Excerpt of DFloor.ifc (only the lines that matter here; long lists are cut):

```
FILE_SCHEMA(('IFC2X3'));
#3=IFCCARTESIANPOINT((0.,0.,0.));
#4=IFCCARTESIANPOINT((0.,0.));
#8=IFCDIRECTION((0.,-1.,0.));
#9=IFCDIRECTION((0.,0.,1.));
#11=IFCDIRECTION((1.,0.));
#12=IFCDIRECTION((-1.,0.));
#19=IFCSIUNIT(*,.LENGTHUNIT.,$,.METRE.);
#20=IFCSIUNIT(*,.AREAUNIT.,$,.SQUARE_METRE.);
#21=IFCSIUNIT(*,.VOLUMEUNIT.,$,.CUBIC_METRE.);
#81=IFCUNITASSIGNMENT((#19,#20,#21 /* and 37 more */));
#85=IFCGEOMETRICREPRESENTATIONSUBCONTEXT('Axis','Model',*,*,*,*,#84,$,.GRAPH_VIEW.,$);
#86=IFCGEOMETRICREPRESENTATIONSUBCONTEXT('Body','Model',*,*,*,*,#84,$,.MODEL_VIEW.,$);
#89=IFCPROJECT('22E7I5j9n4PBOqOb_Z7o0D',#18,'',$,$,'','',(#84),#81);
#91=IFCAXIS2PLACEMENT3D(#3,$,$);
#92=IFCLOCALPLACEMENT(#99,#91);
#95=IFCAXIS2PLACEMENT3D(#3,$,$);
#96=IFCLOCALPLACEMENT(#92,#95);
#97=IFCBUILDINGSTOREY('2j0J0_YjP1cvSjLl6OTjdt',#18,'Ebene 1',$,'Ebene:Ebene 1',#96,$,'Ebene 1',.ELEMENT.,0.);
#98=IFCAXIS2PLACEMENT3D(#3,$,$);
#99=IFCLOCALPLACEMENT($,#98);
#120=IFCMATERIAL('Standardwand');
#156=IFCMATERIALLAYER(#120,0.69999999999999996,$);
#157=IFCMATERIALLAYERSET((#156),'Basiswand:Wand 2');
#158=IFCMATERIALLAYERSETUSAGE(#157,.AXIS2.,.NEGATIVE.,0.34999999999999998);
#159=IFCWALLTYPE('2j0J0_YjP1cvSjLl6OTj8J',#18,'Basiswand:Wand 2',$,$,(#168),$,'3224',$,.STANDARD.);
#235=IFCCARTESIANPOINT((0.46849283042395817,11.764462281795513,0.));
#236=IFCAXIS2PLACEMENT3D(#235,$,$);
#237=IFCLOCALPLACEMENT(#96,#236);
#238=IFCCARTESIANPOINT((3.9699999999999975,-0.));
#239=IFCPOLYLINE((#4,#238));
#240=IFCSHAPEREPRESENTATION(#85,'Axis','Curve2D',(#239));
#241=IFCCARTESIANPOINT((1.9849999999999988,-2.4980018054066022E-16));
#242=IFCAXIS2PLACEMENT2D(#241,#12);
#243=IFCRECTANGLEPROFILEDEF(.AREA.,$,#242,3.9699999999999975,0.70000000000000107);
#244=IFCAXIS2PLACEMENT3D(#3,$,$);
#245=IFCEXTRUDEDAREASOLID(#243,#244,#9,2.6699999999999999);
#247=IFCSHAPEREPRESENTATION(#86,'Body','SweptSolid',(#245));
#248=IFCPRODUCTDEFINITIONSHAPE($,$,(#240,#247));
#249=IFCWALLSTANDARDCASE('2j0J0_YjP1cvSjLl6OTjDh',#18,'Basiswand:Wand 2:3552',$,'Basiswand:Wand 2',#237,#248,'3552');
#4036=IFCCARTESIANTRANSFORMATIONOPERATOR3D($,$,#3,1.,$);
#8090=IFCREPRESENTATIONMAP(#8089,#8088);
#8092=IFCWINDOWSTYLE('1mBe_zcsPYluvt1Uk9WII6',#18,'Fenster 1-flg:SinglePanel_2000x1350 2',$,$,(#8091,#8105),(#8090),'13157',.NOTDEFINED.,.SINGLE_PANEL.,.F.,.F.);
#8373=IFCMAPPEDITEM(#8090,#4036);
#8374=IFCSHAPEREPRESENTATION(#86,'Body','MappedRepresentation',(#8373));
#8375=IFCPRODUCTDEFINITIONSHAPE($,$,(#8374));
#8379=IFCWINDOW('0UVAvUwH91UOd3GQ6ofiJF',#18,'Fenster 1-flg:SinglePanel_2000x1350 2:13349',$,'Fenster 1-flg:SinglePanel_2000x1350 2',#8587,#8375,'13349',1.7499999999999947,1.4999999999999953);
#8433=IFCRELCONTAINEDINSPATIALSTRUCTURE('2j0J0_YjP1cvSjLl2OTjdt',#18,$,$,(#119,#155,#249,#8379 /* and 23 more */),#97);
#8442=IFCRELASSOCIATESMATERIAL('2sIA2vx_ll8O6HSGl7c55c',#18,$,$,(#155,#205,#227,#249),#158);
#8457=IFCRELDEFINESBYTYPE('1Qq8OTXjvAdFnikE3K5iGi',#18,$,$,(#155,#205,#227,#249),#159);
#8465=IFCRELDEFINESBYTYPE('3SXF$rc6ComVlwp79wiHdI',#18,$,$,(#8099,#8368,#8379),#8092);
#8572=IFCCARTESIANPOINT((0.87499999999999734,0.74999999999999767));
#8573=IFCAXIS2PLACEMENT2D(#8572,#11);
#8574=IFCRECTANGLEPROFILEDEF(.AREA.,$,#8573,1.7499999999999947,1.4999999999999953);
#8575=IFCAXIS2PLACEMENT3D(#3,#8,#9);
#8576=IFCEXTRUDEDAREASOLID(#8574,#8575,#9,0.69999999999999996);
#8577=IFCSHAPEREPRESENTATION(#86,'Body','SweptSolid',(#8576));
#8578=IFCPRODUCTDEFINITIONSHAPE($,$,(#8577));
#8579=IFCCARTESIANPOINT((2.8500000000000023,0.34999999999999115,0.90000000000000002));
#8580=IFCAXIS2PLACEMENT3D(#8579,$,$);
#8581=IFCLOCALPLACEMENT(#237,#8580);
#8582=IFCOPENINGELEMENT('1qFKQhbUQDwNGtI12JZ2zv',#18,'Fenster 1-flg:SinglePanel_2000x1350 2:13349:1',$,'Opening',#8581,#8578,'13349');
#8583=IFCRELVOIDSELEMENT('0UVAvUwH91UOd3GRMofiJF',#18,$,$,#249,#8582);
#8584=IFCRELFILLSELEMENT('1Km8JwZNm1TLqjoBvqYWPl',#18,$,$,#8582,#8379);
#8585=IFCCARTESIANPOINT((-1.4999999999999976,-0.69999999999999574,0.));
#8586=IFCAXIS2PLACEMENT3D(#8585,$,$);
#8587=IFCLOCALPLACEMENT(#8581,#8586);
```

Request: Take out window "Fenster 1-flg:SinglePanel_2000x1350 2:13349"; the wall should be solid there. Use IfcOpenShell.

```python
import ifcopenshell
import ifcopenshell.api.feature
import ifcopenshell.api.root
import ifcopenshell.geom
import ifcopenshell.util.shape

model = ifcopenshell.open("DFloor.ifc")
settings = ifcopenshell.geom.settings()


def volume(element):
    """Net volume in cubic metres, openings subtracted."""
    shape = ifcopenshell.geom.create_shape(settings, element)
    return ifcopenshell.util.shape.get_volume(shape.geometry)


window = model.by_guid("0UVAvUwH91UOd3GQ6ofiJF")
opening = window.FillsVoids[0].RelatingOpeningElement
wall = opening.VoidsElements[0].RelatingBuildingElement
before = volume(wall)

ifcopenshell.api.root.remove_product(model, product=window)
ifcopenshell.api.feature.remove_feature(model, feature=opening)

after = volume(wall)

print(f"wall volume {before:.3f} -> {after:.3f} m3")

model.write("DFloor_updated.ifc")
```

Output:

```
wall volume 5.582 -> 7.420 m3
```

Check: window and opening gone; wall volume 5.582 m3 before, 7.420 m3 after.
